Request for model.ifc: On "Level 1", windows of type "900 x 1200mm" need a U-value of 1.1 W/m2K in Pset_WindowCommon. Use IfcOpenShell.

First a look at what the model holds.

```python
import ifcopenshell
import ifcopenshell.util.element

model = ifcopenshell.open("model.ifc")
print(model.schema)
storey = next(s for s in model.by_type("IfcBuildingStorey") if s.Name == "Level 1")
windows = [e for e in ifcopenshell.util.element.get_decomposition(storey) if e.is_a("IfcWindow")]
seen = {}
for e in windows:
    element_type = ifcopenshell.util.element.get_type(e)
    key = (element_type.Name if element_type != e and element_type else None, ifcopenshell.util.element.get_pset(e, "Pset_WindowCommon", "ThermalTransmittance"))
    seen[key] = seen.get(key, 0) + 1
for (name, value), count in sorted(seen.items(), key=str):
    print(count, "x", name, "|", value)
```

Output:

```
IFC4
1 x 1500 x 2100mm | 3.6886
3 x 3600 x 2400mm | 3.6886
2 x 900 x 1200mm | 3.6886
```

```python
import ifcopenshell
import ifcopenshell.api.pset
import ifcopenshell.util.element

model = ifcopenshell.open("model.ifc")

storey = next(s for s in model.by_type("IfcBuildingStorey") if s.Name == "Level 1")
windows = [e for e in ifcopenshell.util.element.get_decomposition(storey) if e.is_a("IfcWindow")]

count = 0
for e in windows:
    element_type = ifcopenshell.util.element.get_type(e)
    if element_type in (None, e) or element_type.Name != "900 x 1200mm":
        continue
    # add_pset returns the element's existing set when there is one.
    pset = ifcopenshell.api.pset.add_pset(model, product=e, name="Pset_WindowCommon")
    ifcopenshell.api.pset.edit_pset(model, pset=pset, properties={"ThermalTransmittance": 1.1})
    count += 1

print(count, "windows updated")

model.write("model_updated.ifc")
```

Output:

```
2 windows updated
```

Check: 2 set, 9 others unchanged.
